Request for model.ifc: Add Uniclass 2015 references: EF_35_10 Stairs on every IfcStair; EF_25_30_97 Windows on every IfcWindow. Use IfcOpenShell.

First a look at what the model holds.

```python
import ifcopenshell

model = ifcopenshell.open("model.ifc")
print(model.schema)
print("classifications:", [c.Name for c in model.by_type("IfcClassification")])
for ifc_class in ("IfcDoor", "IfcRoof", "IfcStair", "IfcWall", "IfcWindow"):
    print(ifc_class, len(model.by_type(ifc_class)))
```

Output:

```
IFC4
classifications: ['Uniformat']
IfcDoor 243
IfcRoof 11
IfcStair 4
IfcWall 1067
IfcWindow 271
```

```python
import ifcopenshell
import ifcopenshell.api.classification

model = ifcopenshell.open("model.ifc")

system = ifcopenshell.api.classification.add_classification(model, classification="Uniclass 2015")

codes = {
    "IfcStair": ("EF_35_10", "Stairs"),
    "IfcWindow": ("EF_25_30_97", "Windows"),
}
for ifc_class, (code, name) in codes.items():
    products = model.by_type(ifc_class)
    ifcopenshell.api.classification.add_reference(
        model, products=products, classification=system, identification=code, name=name
    )
    print(code, len(products))

model.write("model_edited.ifc")
```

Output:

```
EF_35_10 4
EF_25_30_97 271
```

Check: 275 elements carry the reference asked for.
